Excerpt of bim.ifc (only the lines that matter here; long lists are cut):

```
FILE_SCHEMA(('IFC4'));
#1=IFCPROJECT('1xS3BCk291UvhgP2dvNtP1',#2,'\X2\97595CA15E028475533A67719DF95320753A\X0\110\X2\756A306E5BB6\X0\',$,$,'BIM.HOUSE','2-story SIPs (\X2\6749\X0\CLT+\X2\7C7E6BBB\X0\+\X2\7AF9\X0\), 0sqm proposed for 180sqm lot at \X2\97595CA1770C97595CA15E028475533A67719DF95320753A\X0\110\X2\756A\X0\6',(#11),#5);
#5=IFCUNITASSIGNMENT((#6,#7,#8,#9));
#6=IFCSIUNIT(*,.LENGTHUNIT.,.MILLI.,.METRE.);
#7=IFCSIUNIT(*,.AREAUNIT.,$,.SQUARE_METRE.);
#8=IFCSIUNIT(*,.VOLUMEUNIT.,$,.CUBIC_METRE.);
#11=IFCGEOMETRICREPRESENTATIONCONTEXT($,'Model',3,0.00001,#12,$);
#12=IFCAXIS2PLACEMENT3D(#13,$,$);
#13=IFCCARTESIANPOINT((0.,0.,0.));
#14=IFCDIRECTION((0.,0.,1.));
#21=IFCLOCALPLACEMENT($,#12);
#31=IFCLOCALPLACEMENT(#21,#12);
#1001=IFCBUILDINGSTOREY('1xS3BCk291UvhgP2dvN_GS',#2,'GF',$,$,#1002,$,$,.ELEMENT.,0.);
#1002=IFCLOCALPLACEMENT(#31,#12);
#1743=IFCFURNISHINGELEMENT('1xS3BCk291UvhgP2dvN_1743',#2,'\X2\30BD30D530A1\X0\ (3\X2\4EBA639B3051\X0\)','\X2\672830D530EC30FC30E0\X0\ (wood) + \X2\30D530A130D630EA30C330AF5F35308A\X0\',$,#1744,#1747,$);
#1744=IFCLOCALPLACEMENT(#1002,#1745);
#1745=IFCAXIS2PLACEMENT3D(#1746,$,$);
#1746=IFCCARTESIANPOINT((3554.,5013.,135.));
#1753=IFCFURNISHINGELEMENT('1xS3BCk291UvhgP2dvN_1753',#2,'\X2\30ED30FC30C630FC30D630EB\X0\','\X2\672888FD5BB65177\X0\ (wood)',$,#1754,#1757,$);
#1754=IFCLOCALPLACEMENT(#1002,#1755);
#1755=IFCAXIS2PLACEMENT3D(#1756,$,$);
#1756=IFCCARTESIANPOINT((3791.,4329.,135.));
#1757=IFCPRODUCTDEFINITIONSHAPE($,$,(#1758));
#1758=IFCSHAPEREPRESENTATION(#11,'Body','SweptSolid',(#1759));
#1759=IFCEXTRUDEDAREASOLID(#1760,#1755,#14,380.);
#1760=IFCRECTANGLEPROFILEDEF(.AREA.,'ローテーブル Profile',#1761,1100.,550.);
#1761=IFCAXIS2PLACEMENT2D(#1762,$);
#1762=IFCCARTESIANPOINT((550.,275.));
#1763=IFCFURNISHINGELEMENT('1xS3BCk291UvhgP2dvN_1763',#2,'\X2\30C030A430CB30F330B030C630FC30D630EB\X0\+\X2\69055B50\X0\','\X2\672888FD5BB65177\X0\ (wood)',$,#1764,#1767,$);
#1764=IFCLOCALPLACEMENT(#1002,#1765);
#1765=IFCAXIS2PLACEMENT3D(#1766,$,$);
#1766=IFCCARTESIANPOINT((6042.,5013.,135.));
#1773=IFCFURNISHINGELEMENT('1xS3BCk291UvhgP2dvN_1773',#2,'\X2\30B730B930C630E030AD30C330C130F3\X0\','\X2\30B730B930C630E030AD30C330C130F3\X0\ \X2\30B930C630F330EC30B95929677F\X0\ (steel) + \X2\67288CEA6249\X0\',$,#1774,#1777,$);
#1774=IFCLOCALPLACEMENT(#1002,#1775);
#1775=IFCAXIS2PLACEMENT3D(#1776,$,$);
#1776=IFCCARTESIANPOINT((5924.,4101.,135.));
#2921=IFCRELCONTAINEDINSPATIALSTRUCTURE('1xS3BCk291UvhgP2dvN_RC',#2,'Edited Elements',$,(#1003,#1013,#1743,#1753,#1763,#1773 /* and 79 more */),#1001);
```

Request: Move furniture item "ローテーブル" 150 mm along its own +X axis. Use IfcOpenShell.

```python
import ifcopenshell
import ifcopenshell.api.geometry
import ifcopenshell.util.placement

model = ifcopenshell.open("bim.ifc")

item = model.by_guid("1xS3BCk291UvhgP2dvN_1753")
matrix = ifcopenshell.util.placement.get_local_placement(item.ObjectPlacement)
matrix[:3, 3] += matrix[:3, 0] * 150.0
ifcopenshell.api.geometry.edit_object_placement(model, product=item, matrix=matrix, is_si=False)

print(ifcopenshell.util.placement.get_local_placement(item.ObjectPlacement).round(3) + 0.0)

model.write("bim_v2.ifc")
```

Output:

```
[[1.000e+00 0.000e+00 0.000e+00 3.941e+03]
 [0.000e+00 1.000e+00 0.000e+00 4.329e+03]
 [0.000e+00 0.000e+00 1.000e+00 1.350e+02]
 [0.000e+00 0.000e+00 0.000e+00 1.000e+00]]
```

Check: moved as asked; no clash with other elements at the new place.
